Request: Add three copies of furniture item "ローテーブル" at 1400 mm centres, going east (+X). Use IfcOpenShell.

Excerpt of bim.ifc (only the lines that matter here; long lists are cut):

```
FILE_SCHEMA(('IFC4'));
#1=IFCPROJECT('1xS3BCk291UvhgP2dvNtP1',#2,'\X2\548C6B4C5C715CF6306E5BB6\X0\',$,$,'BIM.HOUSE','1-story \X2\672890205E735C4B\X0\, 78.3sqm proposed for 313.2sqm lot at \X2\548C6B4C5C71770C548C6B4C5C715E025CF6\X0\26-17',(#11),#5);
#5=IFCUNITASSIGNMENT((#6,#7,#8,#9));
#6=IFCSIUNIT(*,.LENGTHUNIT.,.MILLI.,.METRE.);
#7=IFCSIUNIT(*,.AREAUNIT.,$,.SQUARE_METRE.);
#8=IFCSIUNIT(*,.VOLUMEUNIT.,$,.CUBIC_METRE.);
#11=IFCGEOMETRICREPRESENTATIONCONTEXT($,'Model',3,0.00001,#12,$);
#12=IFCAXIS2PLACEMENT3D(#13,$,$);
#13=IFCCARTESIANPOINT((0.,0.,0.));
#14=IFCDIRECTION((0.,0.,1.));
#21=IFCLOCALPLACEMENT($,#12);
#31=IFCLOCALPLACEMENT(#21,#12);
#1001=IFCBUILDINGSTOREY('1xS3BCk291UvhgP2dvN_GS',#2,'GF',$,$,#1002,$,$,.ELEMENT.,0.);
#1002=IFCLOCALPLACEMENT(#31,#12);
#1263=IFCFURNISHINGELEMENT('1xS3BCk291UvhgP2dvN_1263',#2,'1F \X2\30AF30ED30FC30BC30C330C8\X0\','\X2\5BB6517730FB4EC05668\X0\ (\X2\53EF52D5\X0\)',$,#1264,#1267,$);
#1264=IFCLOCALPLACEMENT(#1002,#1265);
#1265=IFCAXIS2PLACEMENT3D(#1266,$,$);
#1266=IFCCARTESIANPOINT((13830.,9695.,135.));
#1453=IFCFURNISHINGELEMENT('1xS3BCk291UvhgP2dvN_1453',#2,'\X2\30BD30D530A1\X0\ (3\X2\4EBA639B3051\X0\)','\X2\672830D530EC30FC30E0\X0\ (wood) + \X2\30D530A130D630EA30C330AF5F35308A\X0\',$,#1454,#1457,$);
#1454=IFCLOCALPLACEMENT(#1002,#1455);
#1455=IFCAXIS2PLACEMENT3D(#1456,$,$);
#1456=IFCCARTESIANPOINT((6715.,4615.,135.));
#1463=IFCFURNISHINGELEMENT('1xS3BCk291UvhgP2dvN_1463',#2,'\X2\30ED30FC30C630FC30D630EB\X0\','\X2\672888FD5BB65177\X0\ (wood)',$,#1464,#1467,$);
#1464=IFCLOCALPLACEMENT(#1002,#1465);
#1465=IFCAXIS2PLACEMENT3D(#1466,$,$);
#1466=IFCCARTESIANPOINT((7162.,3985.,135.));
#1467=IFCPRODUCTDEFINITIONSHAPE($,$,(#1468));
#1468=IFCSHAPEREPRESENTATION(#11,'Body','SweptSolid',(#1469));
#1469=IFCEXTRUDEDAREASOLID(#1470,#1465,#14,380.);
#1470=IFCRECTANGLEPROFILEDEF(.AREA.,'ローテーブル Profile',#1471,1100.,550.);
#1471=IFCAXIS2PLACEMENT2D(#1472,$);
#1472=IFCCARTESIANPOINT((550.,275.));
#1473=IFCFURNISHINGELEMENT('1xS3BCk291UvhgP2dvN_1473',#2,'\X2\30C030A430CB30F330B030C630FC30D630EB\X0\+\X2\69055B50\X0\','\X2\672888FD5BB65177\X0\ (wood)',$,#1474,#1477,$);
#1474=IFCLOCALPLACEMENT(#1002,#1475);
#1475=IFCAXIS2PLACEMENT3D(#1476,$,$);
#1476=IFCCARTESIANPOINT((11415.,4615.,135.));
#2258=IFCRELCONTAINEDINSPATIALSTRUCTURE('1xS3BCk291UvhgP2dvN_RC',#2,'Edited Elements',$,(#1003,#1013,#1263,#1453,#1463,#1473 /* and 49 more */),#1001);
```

```python
import numpy as np
import ifcopenshell
import ifcopenshell.api.geometry
import ifcopenshell.api.root
import ifcopenshell.util.element
import ifcopenshell.util.placement

model = ifcopenshell.open("bim.ifc")


def reuse_history(source, copy):
    """copy_class also copies each property set's owner history, people and application; keep the originals."""
    for rel in copy.IsDefinedBy:
        if rel.is_a("IfcRelDefinesByProperties") and (history := rel.RelatingPropertyDefinition.OwnerHistory):
            rel.RelatingPropertyDefinition.OwnerHistory = source.OwnerHistory
            ifcopenshell.util.element.remove_deep2(model, history)


source = model.by_guid("1xS3BCk291UvhgP2dvN_1463")
base = ifcopenshell.util.placement.get_local_placement(source.ObjectPlacement)
step = np.array([1.0, 0.0, 0.0]) * 1400.0

for i in range(1, 4):
    copy = ifcopenshell.api.root.copy_class(model, product=source)
    copy.Representation = ifcopenshell.util.element.copy_deep(
        model, source.Representation, exclude=["IfcGeometricRepresentationContext", "IfcRepresentationMap"]
    )
    reuse_history(source, copy)
    matrix = base.copy()
    matrix[:3, 3] += i * step
    print("added at", matrix[:3, 3].round(3) + 0.0)
    ifcopenshell.api.geometry.edit_object_placement(model, product=copy, matrix=matrix, is_si=False)

model.write("bim_rev.ifc")
```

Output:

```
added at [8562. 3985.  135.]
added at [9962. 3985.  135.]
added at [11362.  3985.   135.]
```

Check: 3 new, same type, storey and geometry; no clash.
